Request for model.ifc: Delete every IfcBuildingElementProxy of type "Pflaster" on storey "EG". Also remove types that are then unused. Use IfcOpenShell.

First a look at what the model holds.

```python
import ifcopenshell
import ifcopenshell.util.element

model = ifcopenshell.open("model.ifc")
print(model.schema)
storey = next(s for s in model.by_type("IfcBuildingStorey") if s.Name == "EG")
proxies = [e for e in ifcopenshell.util.element.get_decomposition(storey) if e.is_a("IfcBuildingElementProxy")]
seen = {}
for e in proxies:
    element_type = ifcopenshell.util.element.get_type(e)
    name = element_type.Name if element_type not in (None, e) else None
    seen[name] = seen.get(name, 0) + 1
for name, count in sorted(seen.items(), key=str):
    print(count, "x", name)
```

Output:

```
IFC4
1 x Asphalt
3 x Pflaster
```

```python
import ifcopenshell
import ifcopenshell.api.root
import ifcopenshell.util.element

model = ifcopenshell.open("model.ifc")

storey = next(s for s in model.by_type("IfcBuildingStorey") if s.Name == "EG")
proxies = [e for e in ifcopenshell.util.element.get_decomposition(storey) if e.is_a("IfcBuildingElementProxy")]
targets = [e for e in proxies if (t := ifcopenshell.util.element.get_type(e)) not in (None, e) and t.Name == "Pflaster"]
types = {ifcopenshell.util.element.get_type(e) for e in targets} - {None, *targets}

for e in targets:
    ifcopenshell.api.root.remove_product(model, product=e)
print(len(targets), "removed")

unused = [t for t in types if not ifcopenshell.util.element.get_types(t)]
for t in unused:
    ifcopenshell.api.root.remove_product(model, product=t)
print(len(unused), "unused types removed")

model.write("model_updated.ifc")
```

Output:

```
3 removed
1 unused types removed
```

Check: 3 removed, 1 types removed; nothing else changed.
